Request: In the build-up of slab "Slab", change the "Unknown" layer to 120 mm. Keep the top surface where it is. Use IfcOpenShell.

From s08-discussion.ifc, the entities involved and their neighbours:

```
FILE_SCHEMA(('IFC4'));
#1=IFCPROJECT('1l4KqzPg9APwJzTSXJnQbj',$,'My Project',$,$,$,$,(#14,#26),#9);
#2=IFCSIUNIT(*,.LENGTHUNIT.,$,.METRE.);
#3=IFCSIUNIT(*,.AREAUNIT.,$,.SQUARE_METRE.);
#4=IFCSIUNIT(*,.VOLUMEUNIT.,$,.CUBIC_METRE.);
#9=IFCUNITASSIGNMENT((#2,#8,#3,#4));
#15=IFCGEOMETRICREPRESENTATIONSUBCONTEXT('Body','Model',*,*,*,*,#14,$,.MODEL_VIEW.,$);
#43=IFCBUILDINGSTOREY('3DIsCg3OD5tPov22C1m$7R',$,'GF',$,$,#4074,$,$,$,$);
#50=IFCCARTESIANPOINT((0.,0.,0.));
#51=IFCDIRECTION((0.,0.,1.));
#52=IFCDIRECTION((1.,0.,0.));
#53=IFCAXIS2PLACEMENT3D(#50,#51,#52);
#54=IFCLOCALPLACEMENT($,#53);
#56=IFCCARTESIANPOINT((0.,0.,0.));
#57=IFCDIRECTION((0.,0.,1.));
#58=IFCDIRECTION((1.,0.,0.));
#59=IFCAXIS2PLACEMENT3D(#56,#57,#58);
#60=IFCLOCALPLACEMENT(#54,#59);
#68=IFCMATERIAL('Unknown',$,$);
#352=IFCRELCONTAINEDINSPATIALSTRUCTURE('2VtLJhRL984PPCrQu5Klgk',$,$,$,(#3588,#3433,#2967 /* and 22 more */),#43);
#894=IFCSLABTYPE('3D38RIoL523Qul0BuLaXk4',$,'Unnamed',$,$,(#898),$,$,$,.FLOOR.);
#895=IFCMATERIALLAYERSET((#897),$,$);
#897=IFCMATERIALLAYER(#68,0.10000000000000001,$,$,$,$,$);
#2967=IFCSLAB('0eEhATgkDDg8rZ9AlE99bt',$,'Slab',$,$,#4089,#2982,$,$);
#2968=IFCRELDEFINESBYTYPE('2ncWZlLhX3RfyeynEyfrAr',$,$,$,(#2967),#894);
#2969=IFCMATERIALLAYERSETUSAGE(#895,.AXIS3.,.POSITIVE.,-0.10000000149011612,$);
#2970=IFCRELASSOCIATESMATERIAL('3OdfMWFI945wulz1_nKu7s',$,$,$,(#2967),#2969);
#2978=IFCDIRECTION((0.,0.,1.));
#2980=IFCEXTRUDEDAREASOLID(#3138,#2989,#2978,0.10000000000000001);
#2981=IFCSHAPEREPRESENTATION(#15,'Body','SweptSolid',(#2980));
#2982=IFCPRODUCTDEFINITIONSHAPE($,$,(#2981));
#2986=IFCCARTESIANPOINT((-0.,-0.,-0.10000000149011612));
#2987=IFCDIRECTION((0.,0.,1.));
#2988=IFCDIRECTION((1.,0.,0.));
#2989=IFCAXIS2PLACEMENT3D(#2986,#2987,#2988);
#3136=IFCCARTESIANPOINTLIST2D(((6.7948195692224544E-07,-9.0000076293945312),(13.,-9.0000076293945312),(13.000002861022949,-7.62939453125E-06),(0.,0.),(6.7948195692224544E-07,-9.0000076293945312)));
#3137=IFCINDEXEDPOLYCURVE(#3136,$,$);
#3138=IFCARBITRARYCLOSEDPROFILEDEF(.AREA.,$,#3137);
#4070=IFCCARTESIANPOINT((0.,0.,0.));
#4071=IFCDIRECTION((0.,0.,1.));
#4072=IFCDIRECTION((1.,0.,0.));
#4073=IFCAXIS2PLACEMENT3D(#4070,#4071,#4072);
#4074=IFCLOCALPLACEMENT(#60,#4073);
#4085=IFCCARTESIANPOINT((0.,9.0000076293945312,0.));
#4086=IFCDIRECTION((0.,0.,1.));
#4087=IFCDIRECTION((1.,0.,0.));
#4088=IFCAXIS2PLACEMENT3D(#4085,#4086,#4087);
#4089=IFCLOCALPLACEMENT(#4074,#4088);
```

```python
import ifcopenshell
import ifcopenshell.util.element
import ifcopenshell.util.representation

model = ifcopenshell.open("s08-discussion.ifc")

layer_set = model.by_id(895)
layer = next(l for l in layer_set.MaterialLayers if l.Material and l.Material.Name == "Unknown")
change = 0.12 - layer.LayerThickness
layer.LayerThickness += change

# Geometry does not follow the layer set by itself.
slabs = [e for e in ifcopenshell.util.element.get_elements_by_material(model, layer_set) if e.is_a("IfcSlab")]
for slab in sorted(slabs, key=lambda e: e.id()):
    body = ifcopenshell.util.representation.get_representation(slab, "Model", "Body")
    solid = body.Items[0]
    old_depth = solid.Depth
    solid.Depth += change
    # Extruded upwards: lower the start of the extrusion so the top stays.
    x, y, z = solid.Position.Location.Coordinates
    solid.Position.Location = model.createIfcCartesianPoint((x, y, z - change))
    print(slab.id(), f"{old_depth:g} -> {solid.Depth:g}")

# The layers are counted up from the underside, which has moved.
for usage in {ifcopenshell.util.element.get_material(slab) for slab in slabs}:
    usage.OffsetFromReferenceLine -= change

model.write("s08-discussion-out.ifc")
```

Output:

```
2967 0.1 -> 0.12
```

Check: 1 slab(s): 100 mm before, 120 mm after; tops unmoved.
